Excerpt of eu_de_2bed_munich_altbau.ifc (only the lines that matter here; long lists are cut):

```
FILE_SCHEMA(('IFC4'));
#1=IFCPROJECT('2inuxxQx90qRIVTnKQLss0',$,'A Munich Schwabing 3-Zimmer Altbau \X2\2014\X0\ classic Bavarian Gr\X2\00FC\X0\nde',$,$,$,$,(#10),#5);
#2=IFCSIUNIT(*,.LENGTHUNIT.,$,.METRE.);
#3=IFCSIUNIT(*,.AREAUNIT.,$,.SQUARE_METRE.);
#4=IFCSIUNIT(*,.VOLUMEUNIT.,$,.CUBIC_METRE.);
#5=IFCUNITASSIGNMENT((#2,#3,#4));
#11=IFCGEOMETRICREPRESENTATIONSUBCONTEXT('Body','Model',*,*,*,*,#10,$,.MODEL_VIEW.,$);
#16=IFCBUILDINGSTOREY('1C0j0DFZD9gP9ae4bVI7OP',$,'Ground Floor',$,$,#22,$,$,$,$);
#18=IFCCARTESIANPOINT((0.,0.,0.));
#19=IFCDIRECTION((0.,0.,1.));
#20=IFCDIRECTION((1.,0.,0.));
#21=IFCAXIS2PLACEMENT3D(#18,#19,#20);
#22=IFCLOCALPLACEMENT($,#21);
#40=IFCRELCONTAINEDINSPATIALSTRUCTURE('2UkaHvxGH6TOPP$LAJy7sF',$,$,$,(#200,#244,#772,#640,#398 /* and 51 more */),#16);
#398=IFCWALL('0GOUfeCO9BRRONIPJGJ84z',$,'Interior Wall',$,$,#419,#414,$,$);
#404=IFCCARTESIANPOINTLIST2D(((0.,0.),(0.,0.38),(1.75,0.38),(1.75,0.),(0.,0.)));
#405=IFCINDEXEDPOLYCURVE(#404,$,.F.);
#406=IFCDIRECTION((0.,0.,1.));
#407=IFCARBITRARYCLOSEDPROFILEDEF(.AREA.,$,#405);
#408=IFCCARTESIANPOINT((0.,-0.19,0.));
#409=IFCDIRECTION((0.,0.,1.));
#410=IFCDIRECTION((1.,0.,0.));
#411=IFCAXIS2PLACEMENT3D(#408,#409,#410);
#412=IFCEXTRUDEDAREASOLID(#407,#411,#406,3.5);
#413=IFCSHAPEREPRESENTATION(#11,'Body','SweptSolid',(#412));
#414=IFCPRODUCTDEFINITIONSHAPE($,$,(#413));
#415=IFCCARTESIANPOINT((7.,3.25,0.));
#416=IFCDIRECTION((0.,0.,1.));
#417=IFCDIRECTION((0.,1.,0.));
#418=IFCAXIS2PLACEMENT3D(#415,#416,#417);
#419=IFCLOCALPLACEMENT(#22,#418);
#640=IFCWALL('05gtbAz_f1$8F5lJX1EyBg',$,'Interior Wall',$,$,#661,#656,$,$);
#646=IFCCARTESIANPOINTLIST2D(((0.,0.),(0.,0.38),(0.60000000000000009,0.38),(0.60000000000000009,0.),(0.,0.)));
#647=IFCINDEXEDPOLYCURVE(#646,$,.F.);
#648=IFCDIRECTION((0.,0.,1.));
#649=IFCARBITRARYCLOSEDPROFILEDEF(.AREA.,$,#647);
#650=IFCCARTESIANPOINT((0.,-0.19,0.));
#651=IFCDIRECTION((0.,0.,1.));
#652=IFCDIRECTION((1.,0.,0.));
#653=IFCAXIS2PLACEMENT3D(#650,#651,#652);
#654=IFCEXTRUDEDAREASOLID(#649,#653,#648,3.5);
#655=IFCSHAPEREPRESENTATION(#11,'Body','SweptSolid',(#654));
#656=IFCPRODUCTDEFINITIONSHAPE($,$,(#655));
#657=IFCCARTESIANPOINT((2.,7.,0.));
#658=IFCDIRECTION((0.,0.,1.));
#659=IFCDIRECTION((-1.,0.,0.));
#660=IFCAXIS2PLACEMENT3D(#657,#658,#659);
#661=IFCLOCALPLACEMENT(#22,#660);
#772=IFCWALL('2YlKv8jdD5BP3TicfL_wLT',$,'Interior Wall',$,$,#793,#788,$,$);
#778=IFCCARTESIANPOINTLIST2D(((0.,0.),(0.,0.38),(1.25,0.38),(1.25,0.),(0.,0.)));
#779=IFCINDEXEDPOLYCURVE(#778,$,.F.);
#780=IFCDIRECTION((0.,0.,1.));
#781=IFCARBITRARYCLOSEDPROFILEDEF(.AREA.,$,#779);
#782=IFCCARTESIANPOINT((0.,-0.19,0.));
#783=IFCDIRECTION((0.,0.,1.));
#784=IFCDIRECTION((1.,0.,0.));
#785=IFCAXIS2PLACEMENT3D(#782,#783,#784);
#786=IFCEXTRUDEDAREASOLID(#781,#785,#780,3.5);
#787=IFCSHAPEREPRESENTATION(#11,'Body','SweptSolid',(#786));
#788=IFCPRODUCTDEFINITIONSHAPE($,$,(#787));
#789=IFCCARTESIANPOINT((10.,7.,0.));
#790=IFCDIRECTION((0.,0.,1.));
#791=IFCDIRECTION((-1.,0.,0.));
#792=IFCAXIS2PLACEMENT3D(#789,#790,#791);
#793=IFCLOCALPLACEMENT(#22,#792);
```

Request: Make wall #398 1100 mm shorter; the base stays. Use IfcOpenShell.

```python
import ifcopenshell
import ifcopenshell.geom
import ifcopenshell.util.representation
import ifcopenshell.util.shape
import ifcopenshell.util.unit

model = ifcopenshell.open("eu_de_2bed_munich_altbau.ifc")
unit_scale = ifcopenshell.util.unit.calculate_unit_scale(model)
settings = ifcopenshell.geom.settings()


def volume(element):
    """Net volume in cubic metres, openings subtracted."""
    shape = ifcopenshell.geom.create_shape(settings, element)
    return ifcopenshell.util.shape.get_volume(shape.geometry)


wall = model.by_guid("0GOUfeCO9BRRONIPJGJ84z")
before = volume(wall)

body = ifcopenshell.util.representation.get_representation(wall, "Model", "Body")
solid = body.Items[0]
old_height = solid.Depth
solid.Depth -= 1.1 / unit_scale
after = volume(wall)

print(f"height {old_height:g} -> {solid.Depth:g}, volume {before:.3f} -> {after:.3f} m3")

model.write("eu_de_2bed_munich_altbau_v2.ifc")
```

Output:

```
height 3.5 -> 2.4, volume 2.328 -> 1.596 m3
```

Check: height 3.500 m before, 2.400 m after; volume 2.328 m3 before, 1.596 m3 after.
